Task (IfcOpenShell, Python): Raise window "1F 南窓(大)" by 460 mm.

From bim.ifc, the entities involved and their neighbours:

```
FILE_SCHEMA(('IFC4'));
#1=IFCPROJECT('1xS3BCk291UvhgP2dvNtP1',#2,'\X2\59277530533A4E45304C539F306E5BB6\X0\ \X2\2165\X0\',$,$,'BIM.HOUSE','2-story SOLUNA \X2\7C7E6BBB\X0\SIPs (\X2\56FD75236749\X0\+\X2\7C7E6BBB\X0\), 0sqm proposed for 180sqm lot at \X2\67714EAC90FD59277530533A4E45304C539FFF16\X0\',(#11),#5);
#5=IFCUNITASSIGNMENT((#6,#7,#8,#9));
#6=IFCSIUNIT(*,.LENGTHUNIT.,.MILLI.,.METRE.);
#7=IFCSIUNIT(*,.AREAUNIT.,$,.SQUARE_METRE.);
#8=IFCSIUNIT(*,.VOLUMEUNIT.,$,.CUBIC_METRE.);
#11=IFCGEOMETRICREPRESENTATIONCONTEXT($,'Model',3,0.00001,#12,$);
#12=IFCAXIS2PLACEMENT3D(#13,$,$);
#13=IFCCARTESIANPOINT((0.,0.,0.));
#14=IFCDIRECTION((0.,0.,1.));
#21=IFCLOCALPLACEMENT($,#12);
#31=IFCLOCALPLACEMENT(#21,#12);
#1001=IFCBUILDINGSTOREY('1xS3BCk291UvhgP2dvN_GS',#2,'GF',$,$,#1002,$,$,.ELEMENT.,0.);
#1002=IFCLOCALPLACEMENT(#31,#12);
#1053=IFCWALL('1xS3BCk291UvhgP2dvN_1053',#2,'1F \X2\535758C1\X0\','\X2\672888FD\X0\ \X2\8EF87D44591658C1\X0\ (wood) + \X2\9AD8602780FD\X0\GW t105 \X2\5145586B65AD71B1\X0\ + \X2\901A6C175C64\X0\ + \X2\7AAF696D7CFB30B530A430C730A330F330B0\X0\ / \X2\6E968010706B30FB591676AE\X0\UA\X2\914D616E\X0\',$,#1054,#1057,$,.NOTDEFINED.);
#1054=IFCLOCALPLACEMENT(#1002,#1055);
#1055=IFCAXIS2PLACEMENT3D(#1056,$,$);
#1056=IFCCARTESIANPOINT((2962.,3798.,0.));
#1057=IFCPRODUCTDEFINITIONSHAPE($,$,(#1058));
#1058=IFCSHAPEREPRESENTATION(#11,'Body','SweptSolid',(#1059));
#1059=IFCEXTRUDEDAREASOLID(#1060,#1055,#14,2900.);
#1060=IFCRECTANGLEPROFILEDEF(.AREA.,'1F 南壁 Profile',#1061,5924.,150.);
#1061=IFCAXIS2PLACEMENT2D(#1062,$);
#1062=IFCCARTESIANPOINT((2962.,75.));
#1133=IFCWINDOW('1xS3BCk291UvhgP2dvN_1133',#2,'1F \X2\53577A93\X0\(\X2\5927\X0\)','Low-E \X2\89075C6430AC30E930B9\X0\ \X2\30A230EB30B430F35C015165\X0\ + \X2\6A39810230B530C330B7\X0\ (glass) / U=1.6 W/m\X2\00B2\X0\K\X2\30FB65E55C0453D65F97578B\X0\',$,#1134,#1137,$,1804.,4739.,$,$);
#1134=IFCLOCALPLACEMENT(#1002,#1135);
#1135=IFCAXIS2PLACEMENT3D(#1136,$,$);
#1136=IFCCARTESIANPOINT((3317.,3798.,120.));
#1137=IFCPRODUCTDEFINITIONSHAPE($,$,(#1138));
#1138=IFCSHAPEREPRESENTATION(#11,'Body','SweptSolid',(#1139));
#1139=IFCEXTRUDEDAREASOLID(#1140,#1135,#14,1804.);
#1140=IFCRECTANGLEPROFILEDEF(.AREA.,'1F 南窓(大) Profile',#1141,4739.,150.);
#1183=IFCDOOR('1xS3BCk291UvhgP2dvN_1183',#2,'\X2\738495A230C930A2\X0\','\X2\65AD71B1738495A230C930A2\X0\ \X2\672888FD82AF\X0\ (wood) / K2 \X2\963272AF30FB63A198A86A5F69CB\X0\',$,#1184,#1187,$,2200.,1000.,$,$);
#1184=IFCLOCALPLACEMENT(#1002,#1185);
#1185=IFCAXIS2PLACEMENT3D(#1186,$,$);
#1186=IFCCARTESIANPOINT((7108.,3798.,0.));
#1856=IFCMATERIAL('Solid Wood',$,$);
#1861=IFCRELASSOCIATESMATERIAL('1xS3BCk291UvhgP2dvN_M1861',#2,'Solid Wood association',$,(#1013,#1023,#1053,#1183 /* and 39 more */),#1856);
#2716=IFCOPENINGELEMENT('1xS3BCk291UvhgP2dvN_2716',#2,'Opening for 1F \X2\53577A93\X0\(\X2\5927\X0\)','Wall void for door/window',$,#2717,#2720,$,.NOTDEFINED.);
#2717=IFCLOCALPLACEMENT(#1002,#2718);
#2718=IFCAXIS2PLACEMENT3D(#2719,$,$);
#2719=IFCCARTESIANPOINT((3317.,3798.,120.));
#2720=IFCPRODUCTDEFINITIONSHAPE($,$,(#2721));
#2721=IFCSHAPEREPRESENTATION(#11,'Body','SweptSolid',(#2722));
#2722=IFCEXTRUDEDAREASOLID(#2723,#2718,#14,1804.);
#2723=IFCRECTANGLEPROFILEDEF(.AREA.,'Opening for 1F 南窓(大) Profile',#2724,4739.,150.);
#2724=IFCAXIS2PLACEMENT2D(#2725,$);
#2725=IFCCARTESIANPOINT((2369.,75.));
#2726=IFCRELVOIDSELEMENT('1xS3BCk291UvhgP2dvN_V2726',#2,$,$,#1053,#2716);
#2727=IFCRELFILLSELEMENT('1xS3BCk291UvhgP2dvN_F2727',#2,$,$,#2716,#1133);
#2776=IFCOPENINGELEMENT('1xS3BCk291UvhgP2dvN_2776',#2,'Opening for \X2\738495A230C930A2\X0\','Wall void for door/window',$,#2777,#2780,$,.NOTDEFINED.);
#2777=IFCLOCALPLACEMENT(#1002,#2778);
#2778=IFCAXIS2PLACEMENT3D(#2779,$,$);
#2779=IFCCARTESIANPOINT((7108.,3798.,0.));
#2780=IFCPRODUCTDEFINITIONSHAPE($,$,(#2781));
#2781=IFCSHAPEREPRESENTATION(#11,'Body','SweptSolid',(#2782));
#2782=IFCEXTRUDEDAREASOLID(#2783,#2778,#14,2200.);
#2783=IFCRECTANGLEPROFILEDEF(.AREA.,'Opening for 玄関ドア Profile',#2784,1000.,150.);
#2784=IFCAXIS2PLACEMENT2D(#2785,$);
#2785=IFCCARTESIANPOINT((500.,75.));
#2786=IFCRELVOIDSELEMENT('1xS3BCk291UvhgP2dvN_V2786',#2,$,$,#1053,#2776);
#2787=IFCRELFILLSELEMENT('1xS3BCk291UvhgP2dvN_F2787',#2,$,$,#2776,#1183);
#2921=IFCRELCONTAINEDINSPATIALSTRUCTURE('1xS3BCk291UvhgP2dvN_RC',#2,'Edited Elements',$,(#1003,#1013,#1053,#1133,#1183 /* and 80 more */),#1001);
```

```python
import numpy as np
import ifcopenshell
import ifcopenshell.api.geometry
import ifcopenshell.util.placement
import ifcopenshell.util.unit

model = ifcopenshell.open("bim.ifc")
unit_scale = ifcopenshell.util.unit.calculate_unit_scale(model)

window = model.by_guid("1xS3BCk291UvhgP2dvN_1133")
opening = window.FillsVoids[0].RelatingOpeningElement
dz = 460.0

shift = np.array([0.0, 0.0, dz])
# The window is not placed relative to its opening, so move both.
for product in (opening, window):
    matrix = ifcopenshell.util.placement.get_local_placement(product.ObjectPlacement)
    matrix[:3, 3] += shift
    ifcopenshell.api.geometry.edit_object_placement(model, product=product, matrix=matrix, is_si=False)

print(f"moved by {dz * unit_scale:+.3f} m")

model.write("bim_v2.ifc")
```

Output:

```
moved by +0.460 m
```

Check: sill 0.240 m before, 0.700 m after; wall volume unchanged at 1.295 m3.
